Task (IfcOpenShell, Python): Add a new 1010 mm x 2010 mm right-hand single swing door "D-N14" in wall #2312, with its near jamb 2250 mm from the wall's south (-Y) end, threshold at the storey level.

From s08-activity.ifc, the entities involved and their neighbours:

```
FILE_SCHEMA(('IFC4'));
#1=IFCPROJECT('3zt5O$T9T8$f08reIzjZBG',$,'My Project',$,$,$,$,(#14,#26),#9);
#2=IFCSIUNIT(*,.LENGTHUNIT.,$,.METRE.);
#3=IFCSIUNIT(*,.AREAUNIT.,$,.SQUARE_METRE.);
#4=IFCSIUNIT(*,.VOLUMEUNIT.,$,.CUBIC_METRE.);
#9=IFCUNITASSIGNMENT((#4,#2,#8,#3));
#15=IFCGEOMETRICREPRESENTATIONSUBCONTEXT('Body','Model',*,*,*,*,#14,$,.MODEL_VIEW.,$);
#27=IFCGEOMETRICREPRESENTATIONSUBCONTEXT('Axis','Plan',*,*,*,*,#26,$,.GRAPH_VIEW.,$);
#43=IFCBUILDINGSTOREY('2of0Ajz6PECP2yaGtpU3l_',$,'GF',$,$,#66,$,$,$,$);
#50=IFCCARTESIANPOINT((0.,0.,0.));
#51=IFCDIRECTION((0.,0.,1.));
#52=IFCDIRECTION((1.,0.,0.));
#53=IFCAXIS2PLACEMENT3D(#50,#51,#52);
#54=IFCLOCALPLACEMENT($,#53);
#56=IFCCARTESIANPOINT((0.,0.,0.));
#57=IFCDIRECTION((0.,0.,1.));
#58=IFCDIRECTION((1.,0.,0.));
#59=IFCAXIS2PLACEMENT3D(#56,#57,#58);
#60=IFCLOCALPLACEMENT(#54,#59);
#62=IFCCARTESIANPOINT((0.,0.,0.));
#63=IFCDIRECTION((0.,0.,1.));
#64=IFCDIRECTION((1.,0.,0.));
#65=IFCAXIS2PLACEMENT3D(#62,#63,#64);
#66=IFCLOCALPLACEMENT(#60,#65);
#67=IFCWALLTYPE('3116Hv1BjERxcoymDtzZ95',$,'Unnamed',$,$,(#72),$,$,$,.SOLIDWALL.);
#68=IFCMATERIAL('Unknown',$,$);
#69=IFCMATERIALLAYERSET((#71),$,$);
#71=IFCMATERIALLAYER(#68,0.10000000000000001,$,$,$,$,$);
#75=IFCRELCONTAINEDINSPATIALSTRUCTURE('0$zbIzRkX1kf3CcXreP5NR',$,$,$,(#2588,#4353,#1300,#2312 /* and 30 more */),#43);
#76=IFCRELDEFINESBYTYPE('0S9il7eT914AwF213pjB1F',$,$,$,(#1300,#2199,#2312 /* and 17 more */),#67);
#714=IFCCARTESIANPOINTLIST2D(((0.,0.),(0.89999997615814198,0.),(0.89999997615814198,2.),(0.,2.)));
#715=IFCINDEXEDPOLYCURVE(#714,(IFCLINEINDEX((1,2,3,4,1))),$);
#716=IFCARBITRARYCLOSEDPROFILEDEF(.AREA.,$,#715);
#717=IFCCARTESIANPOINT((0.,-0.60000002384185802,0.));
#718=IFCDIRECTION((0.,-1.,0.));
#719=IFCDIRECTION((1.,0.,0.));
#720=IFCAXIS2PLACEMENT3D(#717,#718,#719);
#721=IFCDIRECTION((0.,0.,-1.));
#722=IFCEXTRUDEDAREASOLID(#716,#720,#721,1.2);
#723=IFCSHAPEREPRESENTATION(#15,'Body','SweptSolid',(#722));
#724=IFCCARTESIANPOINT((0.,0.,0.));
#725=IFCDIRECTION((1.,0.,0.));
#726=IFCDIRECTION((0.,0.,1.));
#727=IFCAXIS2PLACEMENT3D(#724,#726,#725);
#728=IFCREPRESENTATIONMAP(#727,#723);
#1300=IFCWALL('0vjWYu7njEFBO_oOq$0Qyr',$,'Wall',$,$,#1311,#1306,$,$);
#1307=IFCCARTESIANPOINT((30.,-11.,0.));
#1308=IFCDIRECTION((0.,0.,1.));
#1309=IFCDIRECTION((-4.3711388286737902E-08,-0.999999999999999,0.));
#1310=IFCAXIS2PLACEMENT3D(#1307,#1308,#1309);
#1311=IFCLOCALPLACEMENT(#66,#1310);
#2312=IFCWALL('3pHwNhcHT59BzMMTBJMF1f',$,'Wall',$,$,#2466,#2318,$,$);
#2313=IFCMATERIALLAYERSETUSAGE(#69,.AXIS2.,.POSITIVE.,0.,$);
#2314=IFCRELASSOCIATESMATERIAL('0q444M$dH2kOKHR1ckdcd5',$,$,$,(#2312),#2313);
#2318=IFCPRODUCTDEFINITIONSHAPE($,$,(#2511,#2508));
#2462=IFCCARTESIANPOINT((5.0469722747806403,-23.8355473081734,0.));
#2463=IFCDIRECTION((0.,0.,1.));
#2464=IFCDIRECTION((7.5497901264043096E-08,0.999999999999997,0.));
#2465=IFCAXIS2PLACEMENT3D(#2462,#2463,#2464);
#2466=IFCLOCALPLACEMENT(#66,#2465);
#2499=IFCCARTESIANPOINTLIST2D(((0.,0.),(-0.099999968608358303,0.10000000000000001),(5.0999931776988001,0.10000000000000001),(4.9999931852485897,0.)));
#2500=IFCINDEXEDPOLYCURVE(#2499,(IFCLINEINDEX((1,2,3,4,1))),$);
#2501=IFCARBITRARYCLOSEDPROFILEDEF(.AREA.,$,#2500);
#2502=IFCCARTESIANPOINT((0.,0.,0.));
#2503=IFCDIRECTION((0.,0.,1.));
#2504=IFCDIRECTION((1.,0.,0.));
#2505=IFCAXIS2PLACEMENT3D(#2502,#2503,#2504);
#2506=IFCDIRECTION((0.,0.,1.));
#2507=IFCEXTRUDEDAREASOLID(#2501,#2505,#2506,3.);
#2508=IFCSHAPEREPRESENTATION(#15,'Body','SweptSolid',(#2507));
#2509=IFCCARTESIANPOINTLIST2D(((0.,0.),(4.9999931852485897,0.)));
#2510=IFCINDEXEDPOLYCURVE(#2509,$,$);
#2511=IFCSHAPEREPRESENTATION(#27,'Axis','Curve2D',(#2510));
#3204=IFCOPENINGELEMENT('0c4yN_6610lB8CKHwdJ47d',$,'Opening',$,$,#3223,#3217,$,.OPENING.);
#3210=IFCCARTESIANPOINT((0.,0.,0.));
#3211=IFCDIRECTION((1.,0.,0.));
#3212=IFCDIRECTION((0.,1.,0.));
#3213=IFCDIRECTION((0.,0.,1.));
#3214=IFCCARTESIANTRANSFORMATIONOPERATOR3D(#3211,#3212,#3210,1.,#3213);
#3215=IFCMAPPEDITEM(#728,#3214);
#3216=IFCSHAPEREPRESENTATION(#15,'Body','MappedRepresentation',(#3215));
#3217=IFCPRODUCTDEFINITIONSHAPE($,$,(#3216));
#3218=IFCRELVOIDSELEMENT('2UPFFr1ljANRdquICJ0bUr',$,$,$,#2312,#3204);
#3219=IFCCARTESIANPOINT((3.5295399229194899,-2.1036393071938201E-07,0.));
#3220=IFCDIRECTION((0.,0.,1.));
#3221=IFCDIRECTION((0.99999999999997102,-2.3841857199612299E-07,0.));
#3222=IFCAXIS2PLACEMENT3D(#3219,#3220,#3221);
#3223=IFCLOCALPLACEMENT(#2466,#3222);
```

```python
import numpy as np
import ifcopenshell
import ifcopenshell.api.feature
import ifcopenshell.api.geometry
import ifcopenshell.api.root
import ifcopenshell.api.spatial
import ifcopenshell.geom
import ifcopenshell.util.element
import ifcopenshell.util.placement
import ifcopenshell.util.representation
import ifcopenshell.util.shape
import ifcopenshell.util.unit

model = ifcopenshell.open("s08-activity.ifc")
unit_scale = ifcopenshell.util.unit.calculate_unit_scale(model)
settings = ifcopenshell.geom.settings()


def volume(element):
    """Net volume in cubic metres, openings subtracted."""
    shape = ifcopenshell.geom.create_shape(settings, element)
    return ifcopenshell.util.shape.get_volume(shape.geometry)


wall = model.by_guid("3pHwNhcHT59BzMMTBJMF1f")
storey = ifcopenshell.util.element.get_container(wall, ifc_class="IfcBuildingStorey")
context = ifcopenshell.util.representation.get_context(model, "Model", "Body", "MODEL_VIEW")
before = volume(wall)

width, height, from_end, sill = 1.01, 2.01, 2.25, 0.0  # metres

# The wall runs along its own X axis, and the end named is its -X end.
wall_shape = ifcopenshell.geom.create_shape(settings, wall)
x, y, z = ifcopenshell.util.shape.get_vertices(wall_shape.geometry).T
start = x.min() + from_end
face, thickness = float(y.min()), float(y.max() - y.min())
wall_matrix = ifcopenshell.util.placement.get_local_placement(wall.ObjectPlacement)
level = ifcopenshell.util.placement.get_local_placement(storey.ObjectPlacement)[2, 3]


def in_wall(x, y):
    """Placement at x, y metres in the wall's axes, at sill height."""
    matrix = wall_matrix.copy()
    matrix[:, 3] = wall_matrix @ np.array([x / unit_scale, y / unit_scale, 0.0, 1.0])
    matrix[2, 3] = level + sill / unit_scale
    return matrix


# Opening: a box that overshoots both wall faces by 50 mm.
opening = ifcopenshell.api.root.create_entity(model, ifc_class="IfcOpeningElement", predefined_type="OPENING")
box = ifcopenshell.api.geometry.add_wall_representation(
    model, context=context, length=width, height=height, thickness=thickness + 0.1
)
ifcopenshell.api.geometry.assign_representation(model, product=opening, representation=box)
ifcopenshell.api.geometry.edit_object_placement(model, product=opening, matrix=in_wall(start, face - 0.05), is_si=False)
ifcopenshell.api.feature.add_feature(model, feature=opening, element=wall)

door = ifcopenshell.api.root.create_entity(model, ifc_class="IfcDoor", name="D-N14", predefined_type="DOOR")
door.OverallWidth, door.OverallHeight = width / unit_scale, height / unit_scale
door.OperationType = "SINGLE_SWING_RIGHT"
body = ifcopenshell.api.geometry.add_door_representation(
    model,
    context=context,
    overall_width=door.OverallWidth,
    overall_height=door.OverallHeight,
    operation_type="SINGLE_SWING_RIGHT",
    lining_properties={"LiningDepth": thickness / unit_scale, "ThresholdDepth": thickness / unit_scale},
)
ifcopenshell.api.geometry.assign_representation(model, product=door, representation=body)
ifcopenshell.api.spatial.assign_container(model, products=[door], relating_structure=storey)
ifcopenshell.api.feature.add_filling(model, opening=opening, element=door)

# The lining spans the wall, so the door starts at the wall face.
ifcopenshell.api.geometry.edit_object_placement(model, product=door, matrix=in_wall(start, face), is_si=False)

after = volume(wall)

print(f"wall volume {before:.3f} -> {after:.3f} m3")

model.write("s08-activity_edited.ifc")
```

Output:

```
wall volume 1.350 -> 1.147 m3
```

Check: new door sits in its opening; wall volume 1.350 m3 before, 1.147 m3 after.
